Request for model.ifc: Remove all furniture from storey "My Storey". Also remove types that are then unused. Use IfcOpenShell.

First a look at what the model holds.

```python
import ifcopenshell
import ifcopenshell.util.element

model = ifcopenshell.open("model.ifc")
print(model.schema)
storey = next(s for s in model.by_type("IfcBuildingStorey") if s.Name == "My Storey")
furniture = [e for e in ifcopenshell.util.element.get_decomposition(storey) if e.is_a("IfcFurnishingElement")]
seen = {}
for e in furniture:
    element_type = ifcopenshell.util.element.get_type(e)
    name = element_type.Name if element_type not in (None, e) else None
    seen[name] = seen.get(name, 0) + 1
for name, count in sorted(seen.items(), key=str):
    print(count, "x", name)
```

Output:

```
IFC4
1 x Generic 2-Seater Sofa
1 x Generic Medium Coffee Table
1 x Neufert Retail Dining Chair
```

```python
import ifcopenshell
import ifcopenshell.api.root
import ifcopenshell.util.element

model = ifcopenshell.open("model.ifc")

storey = next(s for s in model.by_type("IfcBuildingStorey") if s.Name == "My Storey")
furniture = [e for e in ifcopenshell.util.element.get_decomposition(storey) if e.is_a("IfcFurnishingElement")]
types = {ifcopenshell.util.element.get_type(e) for e in furniture} - {None, *furniture}

for e in furniture:
    ifcopenshell.api.root.remove_product(model, product=e)
print(len(furniture), "removed")

unused = [t for t in types if not ifcopenshell.util.element.get_types(t)]
for t in unused:
    ifcopenshell.api.root.remove_product(model, product=t)
print(len(unused), "unused types removed")

model.write("model_updated.ifc")
```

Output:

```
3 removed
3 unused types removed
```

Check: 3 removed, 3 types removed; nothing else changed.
